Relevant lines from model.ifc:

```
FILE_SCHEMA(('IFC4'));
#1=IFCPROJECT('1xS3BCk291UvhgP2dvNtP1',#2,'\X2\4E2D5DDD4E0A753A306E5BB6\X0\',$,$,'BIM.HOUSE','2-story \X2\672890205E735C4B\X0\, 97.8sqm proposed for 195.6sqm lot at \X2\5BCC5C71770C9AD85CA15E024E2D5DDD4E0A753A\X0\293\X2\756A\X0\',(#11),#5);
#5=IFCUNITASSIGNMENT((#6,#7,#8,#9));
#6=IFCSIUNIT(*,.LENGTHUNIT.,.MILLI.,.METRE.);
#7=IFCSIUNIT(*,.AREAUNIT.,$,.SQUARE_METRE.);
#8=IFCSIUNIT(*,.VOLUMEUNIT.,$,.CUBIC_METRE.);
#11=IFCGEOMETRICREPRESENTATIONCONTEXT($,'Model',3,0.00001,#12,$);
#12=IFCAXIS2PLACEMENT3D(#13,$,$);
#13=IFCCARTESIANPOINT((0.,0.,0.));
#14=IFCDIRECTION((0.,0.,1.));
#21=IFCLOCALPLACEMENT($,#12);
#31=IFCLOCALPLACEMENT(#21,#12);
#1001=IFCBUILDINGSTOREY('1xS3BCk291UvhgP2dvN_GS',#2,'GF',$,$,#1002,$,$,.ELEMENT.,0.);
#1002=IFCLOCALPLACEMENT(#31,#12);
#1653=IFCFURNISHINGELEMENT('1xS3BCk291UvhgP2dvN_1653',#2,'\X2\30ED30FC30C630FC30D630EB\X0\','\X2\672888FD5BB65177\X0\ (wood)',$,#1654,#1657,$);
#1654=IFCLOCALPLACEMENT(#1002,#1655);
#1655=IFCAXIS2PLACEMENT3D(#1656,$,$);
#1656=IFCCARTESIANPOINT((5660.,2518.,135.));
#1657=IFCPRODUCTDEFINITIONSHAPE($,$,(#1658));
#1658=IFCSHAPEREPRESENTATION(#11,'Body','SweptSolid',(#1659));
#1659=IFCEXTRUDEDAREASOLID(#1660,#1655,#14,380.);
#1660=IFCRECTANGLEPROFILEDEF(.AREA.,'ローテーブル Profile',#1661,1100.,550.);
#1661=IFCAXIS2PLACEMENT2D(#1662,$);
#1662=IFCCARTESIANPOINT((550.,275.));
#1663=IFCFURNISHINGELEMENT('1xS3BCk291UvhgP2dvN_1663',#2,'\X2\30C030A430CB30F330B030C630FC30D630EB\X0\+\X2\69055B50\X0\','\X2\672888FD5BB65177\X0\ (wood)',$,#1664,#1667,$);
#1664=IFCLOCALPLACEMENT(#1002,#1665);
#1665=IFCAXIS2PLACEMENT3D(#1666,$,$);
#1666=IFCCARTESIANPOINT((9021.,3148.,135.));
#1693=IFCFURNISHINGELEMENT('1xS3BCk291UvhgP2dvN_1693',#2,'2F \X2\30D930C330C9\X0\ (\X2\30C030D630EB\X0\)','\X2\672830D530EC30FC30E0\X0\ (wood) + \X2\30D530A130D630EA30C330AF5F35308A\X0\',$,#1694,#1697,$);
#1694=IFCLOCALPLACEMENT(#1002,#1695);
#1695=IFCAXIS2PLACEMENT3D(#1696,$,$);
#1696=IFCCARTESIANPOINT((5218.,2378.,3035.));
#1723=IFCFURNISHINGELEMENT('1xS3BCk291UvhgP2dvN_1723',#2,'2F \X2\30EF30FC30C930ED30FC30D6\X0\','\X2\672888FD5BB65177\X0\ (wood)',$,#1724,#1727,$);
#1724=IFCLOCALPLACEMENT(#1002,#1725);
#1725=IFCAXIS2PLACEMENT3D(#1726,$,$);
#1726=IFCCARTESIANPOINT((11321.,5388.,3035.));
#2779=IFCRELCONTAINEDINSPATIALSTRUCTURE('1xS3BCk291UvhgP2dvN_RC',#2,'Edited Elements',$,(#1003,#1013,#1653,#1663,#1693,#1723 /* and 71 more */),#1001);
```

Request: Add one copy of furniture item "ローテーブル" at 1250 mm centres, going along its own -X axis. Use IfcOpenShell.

```python
import ifcopenshell
import ifcopenshell.api.geometry
import ifcopenshell.api.root
import ifcopenshell.util.element
import ifcopenshell.util.placement
import ifcopenshell.util.unit

model = ifcopenshell.open("model.ifc")
unit_scale = ifcopenshell.util.unit.calculate_unit_scale(model)


def reuse_history(source, copy):
    """copy_class also copies each property set's owner history, people and application; keep the originals."""
    for rel in copy.IsDefinedBy:
        if rel.is_a("IfcRelDefinesByProperties") and (history := rel.RelatingPropertyDefinition.OwnerHistory):
            rel.RelatingPropertyDefinition.OwnerHistory = source.OwnerHistory
            ifcopenshell.util.element.remove_deep2(model, history)


source = model.by_guid("1xS3BCk291UvhgP2dvN_1653")
base = ifcopenshell.util.placement.get_local_placement(source.ObjectPlacement)
step = -base[:3, 0] * 1.25 / unit_scale

for i in range(1, 2):
    copy = ifcopenshell.api.root.copy_class(model, product=source)
    copy.Representation = ifcopenshell.util.element.copy_deep(
        model, source.Representation, exclude=["IfcGeometricRepresentationContext", "IfcRepresentationMap"]
    )
    reuse_history(source, copy)
    matrix = base.copy()
    matrix[:3, 3] += i * step
    print("added at", matrix[:3, 3].round(3) + 0.0)
    ifcopenshell.api.geometry.edit_object_placement(model, product=copy, matrix=matrix, is_si=False)

model.write("model_v2.ifc")
```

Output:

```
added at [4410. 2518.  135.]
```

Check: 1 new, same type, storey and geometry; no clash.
